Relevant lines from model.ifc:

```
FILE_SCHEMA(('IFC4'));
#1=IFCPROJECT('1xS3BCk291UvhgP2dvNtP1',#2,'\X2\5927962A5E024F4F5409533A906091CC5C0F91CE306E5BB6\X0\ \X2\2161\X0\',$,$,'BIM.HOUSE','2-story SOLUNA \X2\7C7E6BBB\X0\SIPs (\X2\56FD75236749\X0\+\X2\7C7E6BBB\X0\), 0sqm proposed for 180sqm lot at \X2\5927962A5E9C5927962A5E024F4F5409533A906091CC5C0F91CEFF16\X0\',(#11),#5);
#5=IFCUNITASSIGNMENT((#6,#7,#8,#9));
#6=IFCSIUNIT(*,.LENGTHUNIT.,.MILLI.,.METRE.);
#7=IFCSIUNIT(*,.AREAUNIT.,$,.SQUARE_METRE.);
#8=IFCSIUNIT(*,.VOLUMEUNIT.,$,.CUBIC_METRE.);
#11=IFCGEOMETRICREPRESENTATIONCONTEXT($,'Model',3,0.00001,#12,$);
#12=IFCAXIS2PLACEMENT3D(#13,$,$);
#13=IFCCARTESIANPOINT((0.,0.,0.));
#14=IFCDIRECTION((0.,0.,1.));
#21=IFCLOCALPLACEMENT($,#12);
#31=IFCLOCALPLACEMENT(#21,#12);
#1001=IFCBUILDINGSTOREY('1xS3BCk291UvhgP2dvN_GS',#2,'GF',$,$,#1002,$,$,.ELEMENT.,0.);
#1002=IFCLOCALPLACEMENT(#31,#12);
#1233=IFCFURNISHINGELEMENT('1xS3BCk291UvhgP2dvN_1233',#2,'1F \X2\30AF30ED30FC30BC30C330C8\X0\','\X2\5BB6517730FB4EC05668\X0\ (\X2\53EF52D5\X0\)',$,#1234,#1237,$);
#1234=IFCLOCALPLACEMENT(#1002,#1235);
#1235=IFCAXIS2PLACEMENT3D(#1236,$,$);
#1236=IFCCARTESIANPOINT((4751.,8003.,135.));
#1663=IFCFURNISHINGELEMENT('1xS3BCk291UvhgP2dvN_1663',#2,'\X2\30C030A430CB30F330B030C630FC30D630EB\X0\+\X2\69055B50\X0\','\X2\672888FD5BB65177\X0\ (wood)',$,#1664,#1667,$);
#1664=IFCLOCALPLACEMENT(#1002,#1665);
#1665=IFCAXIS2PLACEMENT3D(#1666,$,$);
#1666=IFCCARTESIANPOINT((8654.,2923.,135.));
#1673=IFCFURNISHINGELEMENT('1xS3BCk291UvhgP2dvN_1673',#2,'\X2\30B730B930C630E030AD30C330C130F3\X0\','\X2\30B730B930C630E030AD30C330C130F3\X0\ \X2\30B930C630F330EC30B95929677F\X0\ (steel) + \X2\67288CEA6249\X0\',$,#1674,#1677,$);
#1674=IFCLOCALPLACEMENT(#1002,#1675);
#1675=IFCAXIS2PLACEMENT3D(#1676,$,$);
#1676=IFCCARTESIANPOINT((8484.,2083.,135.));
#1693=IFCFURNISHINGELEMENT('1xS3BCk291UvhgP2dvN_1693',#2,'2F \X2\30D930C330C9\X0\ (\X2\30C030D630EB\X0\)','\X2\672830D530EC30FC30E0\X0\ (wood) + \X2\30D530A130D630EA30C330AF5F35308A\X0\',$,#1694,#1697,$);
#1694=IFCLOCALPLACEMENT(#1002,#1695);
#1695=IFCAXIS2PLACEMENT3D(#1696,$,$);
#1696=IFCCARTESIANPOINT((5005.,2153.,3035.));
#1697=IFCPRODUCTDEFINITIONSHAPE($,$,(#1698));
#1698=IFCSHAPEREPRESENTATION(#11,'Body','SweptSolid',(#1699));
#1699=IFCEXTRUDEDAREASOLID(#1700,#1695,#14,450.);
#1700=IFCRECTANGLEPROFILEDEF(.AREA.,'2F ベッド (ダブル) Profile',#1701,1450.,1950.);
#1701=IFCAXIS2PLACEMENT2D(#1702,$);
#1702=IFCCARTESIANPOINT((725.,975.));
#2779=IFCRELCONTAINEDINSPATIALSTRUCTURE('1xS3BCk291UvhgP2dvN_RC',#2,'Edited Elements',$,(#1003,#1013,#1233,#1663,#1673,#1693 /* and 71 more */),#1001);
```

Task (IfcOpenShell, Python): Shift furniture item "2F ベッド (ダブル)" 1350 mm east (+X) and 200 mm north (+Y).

```python
import ifcopenshell
import ifcopenshell.api.geometry
import ifcopenshell.util.placement

model = ifcopenshell.open("model.ifc")

item = model.by_guid("1xS3BCk291UvhgP2dvN_1693")
matrix = ifcopenshell.util.placement.get_local_placement(item.ObjectPlacement)
matrix[0, 3] += 1350.0
matrix[1, 3] += 200.0
ifcopenshell.api.geometry.edit_object_placement(model, product=item, matrix=matrix, is_si=False)

print(ifcopenshell.util.placement.get_local_placement(item.ObjectPlacement).round(3) + 0.0)

model.write("model_edited.ifc")
```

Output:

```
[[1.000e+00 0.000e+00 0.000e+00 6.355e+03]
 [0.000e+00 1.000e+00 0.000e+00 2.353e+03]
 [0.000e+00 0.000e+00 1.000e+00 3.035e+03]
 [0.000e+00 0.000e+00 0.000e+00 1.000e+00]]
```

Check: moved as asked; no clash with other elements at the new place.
